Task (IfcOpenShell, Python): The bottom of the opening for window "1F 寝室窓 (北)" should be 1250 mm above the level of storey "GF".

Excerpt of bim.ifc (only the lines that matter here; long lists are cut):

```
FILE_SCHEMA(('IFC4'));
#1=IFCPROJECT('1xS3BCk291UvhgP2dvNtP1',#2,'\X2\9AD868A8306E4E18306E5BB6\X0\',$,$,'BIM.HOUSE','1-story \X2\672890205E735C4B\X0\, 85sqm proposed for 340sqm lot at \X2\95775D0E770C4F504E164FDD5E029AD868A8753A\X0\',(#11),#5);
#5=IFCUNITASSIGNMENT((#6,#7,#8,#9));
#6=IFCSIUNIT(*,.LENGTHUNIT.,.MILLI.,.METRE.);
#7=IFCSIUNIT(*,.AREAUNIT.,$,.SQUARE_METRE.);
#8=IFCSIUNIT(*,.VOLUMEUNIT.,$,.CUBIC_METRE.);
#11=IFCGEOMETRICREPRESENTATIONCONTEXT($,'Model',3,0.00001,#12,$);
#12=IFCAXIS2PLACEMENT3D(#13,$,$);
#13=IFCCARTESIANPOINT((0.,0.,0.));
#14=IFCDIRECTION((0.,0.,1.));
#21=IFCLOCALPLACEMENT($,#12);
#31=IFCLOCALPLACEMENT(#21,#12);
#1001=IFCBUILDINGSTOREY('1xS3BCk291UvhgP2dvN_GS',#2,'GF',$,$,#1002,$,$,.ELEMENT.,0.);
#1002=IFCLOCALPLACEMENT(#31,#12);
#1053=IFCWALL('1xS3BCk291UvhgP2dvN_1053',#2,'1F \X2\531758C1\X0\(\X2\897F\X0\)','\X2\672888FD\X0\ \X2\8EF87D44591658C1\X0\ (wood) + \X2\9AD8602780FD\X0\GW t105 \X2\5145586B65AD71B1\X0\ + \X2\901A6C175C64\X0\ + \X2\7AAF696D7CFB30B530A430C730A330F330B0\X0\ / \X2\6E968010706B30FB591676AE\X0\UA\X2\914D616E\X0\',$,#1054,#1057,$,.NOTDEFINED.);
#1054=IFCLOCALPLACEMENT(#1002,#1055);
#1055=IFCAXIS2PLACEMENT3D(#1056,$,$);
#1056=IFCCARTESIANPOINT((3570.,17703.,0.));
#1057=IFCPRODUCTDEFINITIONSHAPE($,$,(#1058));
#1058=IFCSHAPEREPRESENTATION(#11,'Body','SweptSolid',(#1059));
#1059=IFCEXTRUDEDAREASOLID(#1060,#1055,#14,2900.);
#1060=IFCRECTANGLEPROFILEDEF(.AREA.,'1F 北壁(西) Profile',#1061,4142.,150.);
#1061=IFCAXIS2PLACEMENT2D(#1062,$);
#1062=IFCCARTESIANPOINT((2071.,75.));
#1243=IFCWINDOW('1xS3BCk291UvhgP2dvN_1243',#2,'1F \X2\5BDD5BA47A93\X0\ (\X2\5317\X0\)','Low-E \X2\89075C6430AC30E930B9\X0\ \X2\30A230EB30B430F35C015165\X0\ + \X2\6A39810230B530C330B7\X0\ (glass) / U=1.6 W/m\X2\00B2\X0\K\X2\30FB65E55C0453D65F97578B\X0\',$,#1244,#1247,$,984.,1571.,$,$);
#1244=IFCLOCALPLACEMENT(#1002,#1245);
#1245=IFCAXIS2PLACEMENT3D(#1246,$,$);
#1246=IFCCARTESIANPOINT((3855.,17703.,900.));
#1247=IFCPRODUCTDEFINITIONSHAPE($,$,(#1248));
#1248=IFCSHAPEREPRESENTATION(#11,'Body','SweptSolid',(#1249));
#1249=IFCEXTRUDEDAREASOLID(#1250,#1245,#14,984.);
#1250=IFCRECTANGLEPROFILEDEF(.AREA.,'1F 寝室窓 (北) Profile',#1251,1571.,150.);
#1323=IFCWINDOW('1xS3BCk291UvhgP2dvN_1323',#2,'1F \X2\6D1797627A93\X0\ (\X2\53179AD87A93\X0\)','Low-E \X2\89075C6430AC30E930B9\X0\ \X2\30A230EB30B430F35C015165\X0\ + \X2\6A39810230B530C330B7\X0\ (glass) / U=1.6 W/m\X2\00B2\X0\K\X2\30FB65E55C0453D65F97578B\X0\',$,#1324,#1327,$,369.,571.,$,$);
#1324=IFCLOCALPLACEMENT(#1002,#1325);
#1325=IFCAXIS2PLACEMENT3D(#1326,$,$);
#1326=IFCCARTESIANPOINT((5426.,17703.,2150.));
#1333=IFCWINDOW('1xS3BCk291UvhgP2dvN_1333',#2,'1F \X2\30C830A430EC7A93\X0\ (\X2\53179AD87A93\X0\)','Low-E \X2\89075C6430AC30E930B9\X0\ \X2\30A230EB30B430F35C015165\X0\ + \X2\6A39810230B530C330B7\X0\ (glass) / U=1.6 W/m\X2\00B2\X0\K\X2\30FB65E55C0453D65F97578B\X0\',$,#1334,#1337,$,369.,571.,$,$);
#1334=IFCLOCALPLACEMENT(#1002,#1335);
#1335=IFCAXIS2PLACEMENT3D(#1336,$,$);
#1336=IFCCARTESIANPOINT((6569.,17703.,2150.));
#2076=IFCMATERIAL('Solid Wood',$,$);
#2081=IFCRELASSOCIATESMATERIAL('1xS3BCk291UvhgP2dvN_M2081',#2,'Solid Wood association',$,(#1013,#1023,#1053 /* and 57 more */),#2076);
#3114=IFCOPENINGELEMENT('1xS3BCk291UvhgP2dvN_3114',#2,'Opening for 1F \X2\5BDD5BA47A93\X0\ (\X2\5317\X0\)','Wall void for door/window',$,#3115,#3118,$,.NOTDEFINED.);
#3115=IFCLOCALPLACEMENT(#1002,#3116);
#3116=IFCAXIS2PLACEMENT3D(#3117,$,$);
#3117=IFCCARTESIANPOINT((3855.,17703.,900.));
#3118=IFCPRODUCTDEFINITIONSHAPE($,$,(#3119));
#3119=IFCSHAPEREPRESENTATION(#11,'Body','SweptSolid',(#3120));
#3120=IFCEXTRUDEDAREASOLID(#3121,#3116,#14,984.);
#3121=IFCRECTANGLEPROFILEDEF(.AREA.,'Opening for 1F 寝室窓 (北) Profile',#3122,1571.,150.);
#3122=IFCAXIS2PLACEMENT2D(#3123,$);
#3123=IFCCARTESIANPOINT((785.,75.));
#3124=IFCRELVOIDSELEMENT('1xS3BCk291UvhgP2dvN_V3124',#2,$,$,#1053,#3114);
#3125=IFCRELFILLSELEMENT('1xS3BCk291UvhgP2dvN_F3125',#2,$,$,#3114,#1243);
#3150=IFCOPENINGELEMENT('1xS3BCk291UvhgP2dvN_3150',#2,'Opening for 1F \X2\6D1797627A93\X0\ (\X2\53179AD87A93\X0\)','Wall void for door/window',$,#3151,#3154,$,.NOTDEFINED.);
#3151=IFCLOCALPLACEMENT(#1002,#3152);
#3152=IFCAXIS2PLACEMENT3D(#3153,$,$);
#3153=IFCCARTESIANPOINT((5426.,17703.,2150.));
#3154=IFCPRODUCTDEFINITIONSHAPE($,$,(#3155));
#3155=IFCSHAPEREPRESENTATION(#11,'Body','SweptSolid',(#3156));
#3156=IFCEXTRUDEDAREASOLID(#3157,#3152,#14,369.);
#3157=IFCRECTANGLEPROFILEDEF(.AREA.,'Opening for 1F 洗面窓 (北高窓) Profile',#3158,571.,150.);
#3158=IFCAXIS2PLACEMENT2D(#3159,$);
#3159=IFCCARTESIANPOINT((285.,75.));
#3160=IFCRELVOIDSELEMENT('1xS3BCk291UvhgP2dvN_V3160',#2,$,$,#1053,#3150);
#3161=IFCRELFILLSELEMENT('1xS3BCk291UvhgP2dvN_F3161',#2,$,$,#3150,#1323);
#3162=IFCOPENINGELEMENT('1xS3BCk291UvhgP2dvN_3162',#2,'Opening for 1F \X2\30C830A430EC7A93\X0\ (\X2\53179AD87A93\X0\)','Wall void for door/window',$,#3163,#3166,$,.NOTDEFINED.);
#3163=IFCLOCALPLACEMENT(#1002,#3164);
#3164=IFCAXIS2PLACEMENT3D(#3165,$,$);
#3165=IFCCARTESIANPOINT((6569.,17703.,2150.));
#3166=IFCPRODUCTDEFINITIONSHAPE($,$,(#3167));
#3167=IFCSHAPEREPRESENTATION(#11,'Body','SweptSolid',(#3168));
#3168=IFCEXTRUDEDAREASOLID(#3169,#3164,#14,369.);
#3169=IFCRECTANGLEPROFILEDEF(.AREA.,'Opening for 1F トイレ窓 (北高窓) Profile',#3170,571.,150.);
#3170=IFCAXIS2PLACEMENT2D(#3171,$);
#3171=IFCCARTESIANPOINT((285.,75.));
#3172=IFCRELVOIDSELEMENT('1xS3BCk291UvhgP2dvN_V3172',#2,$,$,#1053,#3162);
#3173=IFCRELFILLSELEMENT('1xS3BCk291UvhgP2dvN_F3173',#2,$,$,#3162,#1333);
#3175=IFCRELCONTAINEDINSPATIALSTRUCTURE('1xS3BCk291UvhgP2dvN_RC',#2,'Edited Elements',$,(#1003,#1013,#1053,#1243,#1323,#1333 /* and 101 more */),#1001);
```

```python
import numpy as np
import ifcopenshell
import ifcopenshell.api.geometry
import ifcopenshell.geom
import ifcopenshell.util.element
import ifcopenshell.util.placement
import ifcopenshell.util.shape
import ifcopenshell.util.unit

model = ifcopenshell.open("bim.ifc")
unit_scale = ifcopenshell.util.unit.calculate_unit_scale(model)

window = model.by_id(1243)
opening = window.FillsVoids[0].RelatingOpeningElement
storey = ifcopenshell.util.element.get_container(window, ifc_class="IfcBuildingStorey")
level = ifcopenshell.util.placement.get_local_placement(storey.ObjectPlacement)[2, 3]

# The opening's origin need not be at the sill, so measure its lowest point.
shape = ifcopenshell.geom.create_shape(ifcopenshell.geom.settings(), opening)
bottom = ifcopenshell.util.shape.get_shape_bottom_elevation(shape, shape.geometry) / unit_scale
dz = level + 1250.0 - bottom

shift = np.array([0.0, 0.0, dz])
# The window is not placed relative to its opening, so move both.
for product in (opening, window):
    matrix = ifcopenshell.util.placement.get_local_placement(product.ObjectPlacement)
    matrix[:3, 3] += shift
    ifcopenshell.api.geometry.edit_object_placement(model, product=product, matrix=matrix, is_si=False)

print(f"moved by {dz * unit_scale:+.3f} m")

model.write("bim_rev.ifc")
```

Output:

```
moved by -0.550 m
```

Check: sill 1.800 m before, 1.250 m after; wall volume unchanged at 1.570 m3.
